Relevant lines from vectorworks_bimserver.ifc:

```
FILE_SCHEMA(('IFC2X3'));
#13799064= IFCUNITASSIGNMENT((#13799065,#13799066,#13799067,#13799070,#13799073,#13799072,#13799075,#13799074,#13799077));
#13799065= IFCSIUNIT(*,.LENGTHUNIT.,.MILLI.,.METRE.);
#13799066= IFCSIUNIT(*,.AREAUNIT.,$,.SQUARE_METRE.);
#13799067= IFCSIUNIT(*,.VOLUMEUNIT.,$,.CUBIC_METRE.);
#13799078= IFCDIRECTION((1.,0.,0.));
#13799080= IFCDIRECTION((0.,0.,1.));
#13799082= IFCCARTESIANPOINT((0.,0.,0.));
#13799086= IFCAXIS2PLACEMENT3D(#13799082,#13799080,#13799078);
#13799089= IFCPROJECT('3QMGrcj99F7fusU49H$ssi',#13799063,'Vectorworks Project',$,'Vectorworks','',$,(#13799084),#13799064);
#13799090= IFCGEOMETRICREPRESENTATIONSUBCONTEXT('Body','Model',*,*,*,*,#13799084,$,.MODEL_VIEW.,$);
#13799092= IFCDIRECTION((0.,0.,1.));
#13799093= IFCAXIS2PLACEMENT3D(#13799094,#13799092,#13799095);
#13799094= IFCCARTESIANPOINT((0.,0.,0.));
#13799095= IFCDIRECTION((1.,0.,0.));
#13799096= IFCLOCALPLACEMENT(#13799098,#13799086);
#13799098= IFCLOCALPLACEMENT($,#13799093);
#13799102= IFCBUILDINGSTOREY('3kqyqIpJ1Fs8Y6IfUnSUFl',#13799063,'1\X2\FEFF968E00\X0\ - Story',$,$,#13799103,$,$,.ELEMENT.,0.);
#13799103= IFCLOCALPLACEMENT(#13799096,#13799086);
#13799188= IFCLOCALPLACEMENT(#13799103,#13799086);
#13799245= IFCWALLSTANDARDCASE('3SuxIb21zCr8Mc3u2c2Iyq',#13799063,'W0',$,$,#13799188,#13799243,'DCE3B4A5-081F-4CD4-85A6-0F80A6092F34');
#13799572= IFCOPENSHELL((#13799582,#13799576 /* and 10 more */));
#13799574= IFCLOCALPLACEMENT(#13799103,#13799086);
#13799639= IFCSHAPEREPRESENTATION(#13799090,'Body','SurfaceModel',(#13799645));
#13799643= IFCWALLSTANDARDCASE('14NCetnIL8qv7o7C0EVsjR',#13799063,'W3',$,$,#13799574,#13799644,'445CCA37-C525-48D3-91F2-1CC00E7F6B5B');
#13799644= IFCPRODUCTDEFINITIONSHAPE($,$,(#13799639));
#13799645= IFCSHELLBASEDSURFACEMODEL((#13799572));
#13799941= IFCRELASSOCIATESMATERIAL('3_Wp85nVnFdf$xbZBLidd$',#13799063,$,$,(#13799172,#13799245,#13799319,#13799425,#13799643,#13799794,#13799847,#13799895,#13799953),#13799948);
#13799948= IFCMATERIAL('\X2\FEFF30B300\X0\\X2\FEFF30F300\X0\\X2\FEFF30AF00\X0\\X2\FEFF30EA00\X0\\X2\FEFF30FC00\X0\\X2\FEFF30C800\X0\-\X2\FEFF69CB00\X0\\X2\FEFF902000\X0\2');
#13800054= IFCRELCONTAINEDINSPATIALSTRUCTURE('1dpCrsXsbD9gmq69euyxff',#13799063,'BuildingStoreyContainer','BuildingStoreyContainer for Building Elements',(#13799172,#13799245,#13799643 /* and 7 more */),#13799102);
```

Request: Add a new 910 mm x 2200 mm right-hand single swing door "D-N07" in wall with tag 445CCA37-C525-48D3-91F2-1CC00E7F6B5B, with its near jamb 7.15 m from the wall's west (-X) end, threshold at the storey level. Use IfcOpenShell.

```python
import numpy as np
import ifcopenshell
import ifcopenshell.api.feature
import ifcopenshell.api.geometry
import ifcopenshell.api.root
import ifcopenshell.api.spatial
import ifcopenshell.api.type
import ifcopenshell.geom
import ifcopenshell.util.element
import ifcopenshell.util.placement
import ifcopenshell.util.representation
import ifcopenshell.util.shape
import ifcopenshell.util.unit

model = ifcopenshell.open("vectorworks_bimserver.ifc")
unit_scale = ifcopenshell.util.unit.calculate_unit_scale(model)
settings = ifcopenshell.geom.settings()


def volume(element):
    """Net volume in cubic metres, openings subtracted."""
    shape = ifcopenshell.geom.create_shape(settings, element)
    return ifcopenshell.util.shape.get_volume(shape.geometry)


wall = model.by_id(13799643)
storey = ifcopenshell.util.element.get_container(wall, ifc_class="IfcBuildingStorey")
context = ifcopenshell.util.representation.get_context(model, "Model", "Body", "MODEL_VIEW")
before = volume(wall)

width, height, from_end, sill = 0.91, 2.2, 7.15, 0.0  # metres

# The wall runs along its own X axis, and the end named is its -X end.
wall_shape = ifcopenshell.geom.create_shape(settings, wall)
x, y, z = ifcopenshell.util.shape.get_vertices(wall_shape.geometry).T
start = x.min() + from_end
face, thickness = float(y.min()), float(y.max() - y.min())
wall_matrix = ifcopenshell.util.placement.get_local_placement(wall.ObjectPlacement)
level = ifcopenshell.util.placement.get_local_placement(storey.ObjectPlacement)[2, 3]


def in_wall(x, y):
    """Placement at x, y metres in the wall's axes, at sill height."""
    matrix = wall_matrix.copy()
    matrix[:, 3] = wall_matrix @ np.array([x / unit_scale, y / unit_scale, 0.0, 1.0])
    matrix[2, 3] = level + sill / unit_scale
    return matrix


# Opening: a box that overshoots both wall faces by 50 mm.
opening = ifcopenshell.api.root.create_entity(model, ifc_class="IfcOpeningElement")
box = ifcopenshell.api.geometry.add_wall_representation(
    model, context=context, length=width, height=height, thickness=thickness + 0.1
)
ifcopenshell.api.geometry.assign_representation(model, product=opening, representation=box)
ifcopenshell.api.geometry.edit_object_placement(model, product=opening, matrix=in_wall(start, face - 0.05), is_si=False)
ifcopenshell.api.feature.add_feature(model, feature=opening, element=wall)

door = ifcopenshell.api.root.create_entity(model, ifc_class="IfcDoor", name="D-N07")
door.OverallWidth, door.OverallHeight = width / unit_scale, height / unit_scale
body = ifcopenshell.api.geometry.add_door_representation(
    model,
    context=context,
    overall_width=door.OverallWidth,
    overall_height=door.OverallHeight,
    operation_type="SINGLE_SWING_RIGHT",
    lining_properties={"LiningDepth": thickness / unit_scale, "ThresholdDepth": thickness / unit_scale},
)
ifcopenshell.api.geometry.assign_representation(model, product=door, representation=body)
ifcopenshell.api.spatial.assign_container(model, products=[door], relating_structure=storey)
fills = ifcopenshell.api.feature.add_filling(model, opening=opening, element=door)
fills.OwnerHistory = door.OwnerHistory  # required in IFC2X3

# IFC2X3 keeps the operation on the door style.
style = ifcopenshell.api.root.create_entity(model, ifc_class="IfcDoorStyle", name="D-N07")
style.OperationType, style.ConstructionType = "SINGLE_SWING_RIGHT", "NOTDEFINED"
style.ParameterTakesPrecedence = style.Sizeable = False
ifcopenshell.api.type.assign_type(model, related_objects=[door], relating_type=style)

# The lining spans the wall, so the door starts at the wall face.
ifcopenshell.api.geometry.edit_object_placement(model, product=door, matrix=in_wall(start, face), is_si=False)

after = volume(wall)

print(f"wall volume {before:.3f} -> {after:.3f} m3")

model.write("vectorworks_bimserver_edited.ifc")
```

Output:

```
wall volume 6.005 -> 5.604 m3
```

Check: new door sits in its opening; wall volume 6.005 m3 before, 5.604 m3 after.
